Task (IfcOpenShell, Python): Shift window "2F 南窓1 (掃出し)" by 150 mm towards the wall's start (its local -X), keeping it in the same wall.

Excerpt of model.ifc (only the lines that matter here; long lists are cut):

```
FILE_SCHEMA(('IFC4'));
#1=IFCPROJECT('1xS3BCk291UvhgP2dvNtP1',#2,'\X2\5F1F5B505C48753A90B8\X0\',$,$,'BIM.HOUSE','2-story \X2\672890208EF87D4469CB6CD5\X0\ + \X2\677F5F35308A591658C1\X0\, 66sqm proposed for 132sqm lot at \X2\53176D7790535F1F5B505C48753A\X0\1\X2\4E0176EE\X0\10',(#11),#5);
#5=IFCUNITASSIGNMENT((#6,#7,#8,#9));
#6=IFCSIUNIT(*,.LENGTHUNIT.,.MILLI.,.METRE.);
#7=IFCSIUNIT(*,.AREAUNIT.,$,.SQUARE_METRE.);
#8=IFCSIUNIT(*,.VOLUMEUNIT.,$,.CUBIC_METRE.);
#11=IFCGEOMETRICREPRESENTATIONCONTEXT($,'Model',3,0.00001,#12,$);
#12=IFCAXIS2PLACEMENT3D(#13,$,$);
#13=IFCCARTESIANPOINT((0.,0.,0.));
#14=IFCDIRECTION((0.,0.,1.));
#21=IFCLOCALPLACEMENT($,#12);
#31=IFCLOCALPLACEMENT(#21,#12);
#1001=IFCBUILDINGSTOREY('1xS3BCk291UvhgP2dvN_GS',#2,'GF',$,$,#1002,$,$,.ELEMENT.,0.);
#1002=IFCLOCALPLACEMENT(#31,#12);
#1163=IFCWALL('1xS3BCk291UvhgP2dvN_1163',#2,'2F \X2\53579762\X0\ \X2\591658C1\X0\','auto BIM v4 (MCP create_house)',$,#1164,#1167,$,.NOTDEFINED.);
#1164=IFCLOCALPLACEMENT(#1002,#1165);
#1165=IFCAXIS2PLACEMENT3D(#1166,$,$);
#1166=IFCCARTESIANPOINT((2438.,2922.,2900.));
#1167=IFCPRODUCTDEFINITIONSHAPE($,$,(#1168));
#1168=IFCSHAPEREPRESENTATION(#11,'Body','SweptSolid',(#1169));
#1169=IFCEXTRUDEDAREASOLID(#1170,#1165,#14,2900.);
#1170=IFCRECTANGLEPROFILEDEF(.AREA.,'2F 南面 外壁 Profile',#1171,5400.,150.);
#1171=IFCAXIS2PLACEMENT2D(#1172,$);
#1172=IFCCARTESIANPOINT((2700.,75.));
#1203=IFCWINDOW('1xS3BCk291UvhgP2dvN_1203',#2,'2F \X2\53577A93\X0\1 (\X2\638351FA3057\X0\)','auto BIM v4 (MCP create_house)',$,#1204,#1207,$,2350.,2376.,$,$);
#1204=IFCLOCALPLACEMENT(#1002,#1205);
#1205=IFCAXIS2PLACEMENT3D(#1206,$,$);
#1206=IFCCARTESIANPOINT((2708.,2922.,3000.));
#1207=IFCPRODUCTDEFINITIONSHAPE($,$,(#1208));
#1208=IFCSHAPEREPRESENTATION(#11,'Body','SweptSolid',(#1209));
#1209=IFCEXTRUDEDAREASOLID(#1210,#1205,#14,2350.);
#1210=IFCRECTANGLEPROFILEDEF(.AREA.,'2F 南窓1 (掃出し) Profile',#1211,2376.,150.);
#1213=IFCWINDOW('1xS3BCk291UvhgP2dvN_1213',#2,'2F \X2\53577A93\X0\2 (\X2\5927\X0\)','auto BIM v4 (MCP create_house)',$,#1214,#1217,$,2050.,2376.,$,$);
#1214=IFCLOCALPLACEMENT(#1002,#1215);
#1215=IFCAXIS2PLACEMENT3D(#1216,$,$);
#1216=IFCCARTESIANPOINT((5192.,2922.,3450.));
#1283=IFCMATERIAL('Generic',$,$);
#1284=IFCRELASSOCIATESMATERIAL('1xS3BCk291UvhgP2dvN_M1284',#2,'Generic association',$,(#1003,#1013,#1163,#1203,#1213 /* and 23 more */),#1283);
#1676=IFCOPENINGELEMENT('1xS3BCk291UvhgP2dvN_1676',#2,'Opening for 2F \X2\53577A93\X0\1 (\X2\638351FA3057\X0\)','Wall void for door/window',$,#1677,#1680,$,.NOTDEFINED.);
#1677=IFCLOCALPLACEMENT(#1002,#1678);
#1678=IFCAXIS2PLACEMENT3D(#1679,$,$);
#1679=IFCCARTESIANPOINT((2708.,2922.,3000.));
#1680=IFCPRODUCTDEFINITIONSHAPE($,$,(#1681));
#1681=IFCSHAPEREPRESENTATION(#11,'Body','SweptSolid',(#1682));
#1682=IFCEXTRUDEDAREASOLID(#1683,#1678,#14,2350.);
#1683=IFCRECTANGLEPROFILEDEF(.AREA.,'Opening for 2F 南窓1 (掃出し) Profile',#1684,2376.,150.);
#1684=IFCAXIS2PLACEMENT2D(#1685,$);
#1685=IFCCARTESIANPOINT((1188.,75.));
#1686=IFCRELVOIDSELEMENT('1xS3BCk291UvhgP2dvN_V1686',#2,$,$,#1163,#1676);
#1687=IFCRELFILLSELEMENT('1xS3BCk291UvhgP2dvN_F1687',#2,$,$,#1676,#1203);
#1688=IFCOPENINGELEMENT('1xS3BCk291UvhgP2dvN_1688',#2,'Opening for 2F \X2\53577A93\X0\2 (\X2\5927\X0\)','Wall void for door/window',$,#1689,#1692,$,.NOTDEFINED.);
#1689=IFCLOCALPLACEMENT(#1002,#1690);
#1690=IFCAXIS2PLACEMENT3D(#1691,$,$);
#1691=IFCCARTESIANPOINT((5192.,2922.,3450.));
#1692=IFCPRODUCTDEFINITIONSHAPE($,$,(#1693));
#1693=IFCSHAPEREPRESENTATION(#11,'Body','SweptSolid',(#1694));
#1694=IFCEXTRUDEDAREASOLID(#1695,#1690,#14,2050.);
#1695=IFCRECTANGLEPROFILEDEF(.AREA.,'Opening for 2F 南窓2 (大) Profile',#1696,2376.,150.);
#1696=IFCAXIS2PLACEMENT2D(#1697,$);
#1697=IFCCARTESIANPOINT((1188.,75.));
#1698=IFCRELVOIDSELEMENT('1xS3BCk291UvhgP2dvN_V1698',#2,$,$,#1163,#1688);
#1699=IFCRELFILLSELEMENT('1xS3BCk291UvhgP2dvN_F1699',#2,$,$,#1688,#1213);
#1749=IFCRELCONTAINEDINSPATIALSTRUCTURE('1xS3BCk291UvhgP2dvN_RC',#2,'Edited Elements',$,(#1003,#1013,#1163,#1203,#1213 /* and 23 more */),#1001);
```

```python
import ifcopenshell
import ifcopenshell.api.geometry
import ifcopenshell.util.placement
import ifcopenshell.util.unit

model = ifcopenshell.open("model.ifc")
unit_scale = ifcopenshell.util.unit.calculate_unit_scale(model)

window = model.by_guid("1xS3BCk291UvhgP2dvN_1203")
opening = window.FillsVoids[0].RelatingOpeningElement
wall = opening.VoidsElements[0].RelatingBuildingElement

wall_matrix = ifcopenshell.util.placement.get_local_placement(wall.ObjectPlacement)
shift = wall_matrix[:3, 0] * -0.15 / unit_scale
before = ifcopenshell.util.placement.get_local_placement(window.ObjectPlacement)[:3, 3].copy()

# The window is not placed relative to its opening, so move both.
for product in (opening, window):
    matrix = ifcopenshell.util.placement.get_local_placement(product.ObjectPlacement)
    matrix[:3, 3] += shift
    ifcopenshell.api.geometry.edit_object_placement(model, product=product, matrix=matrix, is_si=False)

after = ifcopenshell.util.placement.get_local_placement(window.ObjectPlacement)[:3, 3]
print("window moved by", (after - before).round(3) + 0.0)

model.write("model_updated.ifc")
```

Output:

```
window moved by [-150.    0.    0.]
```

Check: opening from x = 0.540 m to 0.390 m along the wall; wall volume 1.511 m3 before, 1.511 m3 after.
